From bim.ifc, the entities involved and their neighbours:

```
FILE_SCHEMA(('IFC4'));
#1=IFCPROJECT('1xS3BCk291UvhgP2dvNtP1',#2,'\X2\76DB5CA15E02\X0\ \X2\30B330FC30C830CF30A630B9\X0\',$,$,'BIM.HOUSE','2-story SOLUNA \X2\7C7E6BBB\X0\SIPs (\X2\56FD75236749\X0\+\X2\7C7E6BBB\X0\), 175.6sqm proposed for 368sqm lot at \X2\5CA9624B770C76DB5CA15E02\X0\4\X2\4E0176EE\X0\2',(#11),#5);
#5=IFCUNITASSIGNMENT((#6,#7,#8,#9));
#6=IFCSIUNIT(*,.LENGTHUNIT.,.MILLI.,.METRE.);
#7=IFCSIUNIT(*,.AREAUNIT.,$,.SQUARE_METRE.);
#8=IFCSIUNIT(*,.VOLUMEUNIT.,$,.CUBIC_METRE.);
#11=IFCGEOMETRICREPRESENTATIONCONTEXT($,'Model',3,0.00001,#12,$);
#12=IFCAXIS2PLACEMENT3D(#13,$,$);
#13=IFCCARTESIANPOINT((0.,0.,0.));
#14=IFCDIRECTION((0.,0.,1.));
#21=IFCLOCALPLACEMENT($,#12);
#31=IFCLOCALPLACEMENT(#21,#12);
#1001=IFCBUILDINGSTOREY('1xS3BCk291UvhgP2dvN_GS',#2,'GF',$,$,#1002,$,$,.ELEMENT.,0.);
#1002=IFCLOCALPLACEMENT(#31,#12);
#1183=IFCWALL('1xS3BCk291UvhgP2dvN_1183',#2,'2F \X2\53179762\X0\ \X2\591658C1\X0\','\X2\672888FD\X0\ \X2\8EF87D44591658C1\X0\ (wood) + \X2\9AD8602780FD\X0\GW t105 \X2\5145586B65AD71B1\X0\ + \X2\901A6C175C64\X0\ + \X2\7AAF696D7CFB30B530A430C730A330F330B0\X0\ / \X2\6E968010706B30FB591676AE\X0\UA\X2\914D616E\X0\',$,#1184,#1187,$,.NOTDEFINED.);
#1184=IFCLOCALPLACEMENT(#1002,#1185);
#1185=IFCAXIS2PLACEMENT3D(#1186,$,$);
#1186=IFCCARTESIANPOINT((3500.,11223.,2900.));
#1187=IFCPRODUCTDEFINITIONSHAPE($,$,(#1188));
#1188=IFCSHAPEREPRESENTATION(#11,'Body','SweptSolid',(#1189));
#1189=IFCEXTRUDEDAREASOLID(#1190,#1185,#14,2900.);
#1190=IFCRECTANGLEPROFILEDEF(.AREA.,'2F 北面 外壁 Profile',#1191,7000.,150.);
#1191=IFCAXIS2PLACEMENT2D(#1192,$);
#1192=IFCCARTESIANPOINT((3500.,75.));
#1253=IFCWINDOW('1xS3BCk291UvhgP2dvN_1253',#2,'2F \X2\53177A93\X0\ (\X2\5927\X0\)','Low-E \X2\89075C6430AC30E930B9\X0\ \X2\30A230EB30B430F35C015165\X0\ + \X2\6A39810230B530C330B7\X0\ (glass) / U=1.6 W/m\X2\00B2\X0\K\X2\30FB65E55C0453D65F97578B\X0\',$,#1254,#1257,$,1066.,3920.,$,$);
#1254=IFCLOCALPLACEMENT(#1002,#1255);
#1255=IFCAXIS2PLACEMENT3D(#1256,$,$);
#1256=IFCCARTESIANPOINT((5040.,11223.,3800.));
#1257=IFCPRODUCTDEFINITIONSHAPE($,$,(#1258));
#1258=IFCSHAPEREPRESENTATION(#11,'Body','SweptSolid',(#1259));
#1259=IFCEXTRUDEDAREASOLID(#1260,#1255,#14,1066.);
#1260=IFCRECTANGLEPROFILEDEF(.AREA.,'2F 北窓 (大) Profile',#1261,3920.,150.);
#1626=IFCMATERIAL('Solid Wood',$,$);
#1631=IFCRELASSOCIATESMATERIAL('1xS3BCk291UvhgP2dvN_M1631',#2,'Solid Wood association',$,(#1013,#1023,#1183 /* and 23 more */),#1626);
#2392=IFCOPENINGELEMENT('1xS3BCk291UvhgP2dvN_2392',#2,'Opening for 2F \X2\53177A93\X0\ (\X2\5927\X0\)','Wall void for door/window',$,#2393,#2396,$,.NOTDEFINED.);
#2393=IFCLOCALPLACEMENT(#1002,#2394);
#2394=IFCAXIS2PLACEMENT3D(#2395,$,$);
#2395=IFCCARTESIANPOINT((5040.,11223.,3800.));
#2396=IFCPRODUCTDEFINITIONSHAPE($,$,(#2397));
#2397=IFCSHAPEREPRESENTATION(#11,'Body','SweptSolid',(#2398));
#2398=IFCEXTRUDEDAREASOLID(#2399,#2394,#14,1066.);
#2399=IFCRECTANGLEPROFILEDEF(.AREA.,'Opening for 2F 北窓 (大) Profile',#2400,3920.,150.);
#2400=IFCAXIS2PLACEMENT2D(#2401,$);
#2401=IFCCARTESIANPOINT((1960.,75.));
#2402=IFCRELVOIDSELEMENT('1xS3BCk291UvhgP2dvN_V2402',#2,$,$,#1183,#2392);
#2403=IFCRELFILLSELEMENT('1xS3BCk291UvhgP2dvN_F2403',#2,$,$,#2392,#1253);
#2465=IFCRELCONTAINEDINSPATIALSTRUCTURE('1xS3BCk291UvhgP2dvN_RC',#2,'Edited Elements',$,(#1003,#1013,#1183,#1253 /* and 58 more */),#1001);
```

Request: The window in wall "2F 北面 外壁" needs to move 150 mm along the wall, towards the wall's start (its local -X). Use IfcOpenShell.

```python
import ifcopenshell
import ifcopenshell.api.geometry
import ifcopenshell.util.placement

model = ifcopenshell.open("bim.ifc")

window = model.by_id(1253)
opening = window.FillsVoids[0].RelatingOpeningElement
wall = opening.VoidsElements[0].RelatingBuildingElement

wall_matrix = ifcopenshell.util.placement.get_local_placement(wall.ObjectPlacement)
shift = wall_matrix[:3, 0] * -150.0
before = ifcopenshell.util.placement.get_local_placement(window.ObjectPlacement)[:3, 3].copy()

# The window is not placed relative to its opening, so move both.
for product in (opening, window):
    matrix = ifcopenshell.util.placement.get_local_placement(product.ObjectPlacement)
    matrix[:3, 3] += shift
    ifcopenshell.api.geometry.edit_object_placement(model, product=product, matrix=matrix, is_si=False)

after = ifcopenshell.util.placement.get_local_placement(window.ObjectPlacement)[:3, 3]
print("window moved by", (after - before).round(3) + 0.0)

model.write("bim_rev.ifc")
```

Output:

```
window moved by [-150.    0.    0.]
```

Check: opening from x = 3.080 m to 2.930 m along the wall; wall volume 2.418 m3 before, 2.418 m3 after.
